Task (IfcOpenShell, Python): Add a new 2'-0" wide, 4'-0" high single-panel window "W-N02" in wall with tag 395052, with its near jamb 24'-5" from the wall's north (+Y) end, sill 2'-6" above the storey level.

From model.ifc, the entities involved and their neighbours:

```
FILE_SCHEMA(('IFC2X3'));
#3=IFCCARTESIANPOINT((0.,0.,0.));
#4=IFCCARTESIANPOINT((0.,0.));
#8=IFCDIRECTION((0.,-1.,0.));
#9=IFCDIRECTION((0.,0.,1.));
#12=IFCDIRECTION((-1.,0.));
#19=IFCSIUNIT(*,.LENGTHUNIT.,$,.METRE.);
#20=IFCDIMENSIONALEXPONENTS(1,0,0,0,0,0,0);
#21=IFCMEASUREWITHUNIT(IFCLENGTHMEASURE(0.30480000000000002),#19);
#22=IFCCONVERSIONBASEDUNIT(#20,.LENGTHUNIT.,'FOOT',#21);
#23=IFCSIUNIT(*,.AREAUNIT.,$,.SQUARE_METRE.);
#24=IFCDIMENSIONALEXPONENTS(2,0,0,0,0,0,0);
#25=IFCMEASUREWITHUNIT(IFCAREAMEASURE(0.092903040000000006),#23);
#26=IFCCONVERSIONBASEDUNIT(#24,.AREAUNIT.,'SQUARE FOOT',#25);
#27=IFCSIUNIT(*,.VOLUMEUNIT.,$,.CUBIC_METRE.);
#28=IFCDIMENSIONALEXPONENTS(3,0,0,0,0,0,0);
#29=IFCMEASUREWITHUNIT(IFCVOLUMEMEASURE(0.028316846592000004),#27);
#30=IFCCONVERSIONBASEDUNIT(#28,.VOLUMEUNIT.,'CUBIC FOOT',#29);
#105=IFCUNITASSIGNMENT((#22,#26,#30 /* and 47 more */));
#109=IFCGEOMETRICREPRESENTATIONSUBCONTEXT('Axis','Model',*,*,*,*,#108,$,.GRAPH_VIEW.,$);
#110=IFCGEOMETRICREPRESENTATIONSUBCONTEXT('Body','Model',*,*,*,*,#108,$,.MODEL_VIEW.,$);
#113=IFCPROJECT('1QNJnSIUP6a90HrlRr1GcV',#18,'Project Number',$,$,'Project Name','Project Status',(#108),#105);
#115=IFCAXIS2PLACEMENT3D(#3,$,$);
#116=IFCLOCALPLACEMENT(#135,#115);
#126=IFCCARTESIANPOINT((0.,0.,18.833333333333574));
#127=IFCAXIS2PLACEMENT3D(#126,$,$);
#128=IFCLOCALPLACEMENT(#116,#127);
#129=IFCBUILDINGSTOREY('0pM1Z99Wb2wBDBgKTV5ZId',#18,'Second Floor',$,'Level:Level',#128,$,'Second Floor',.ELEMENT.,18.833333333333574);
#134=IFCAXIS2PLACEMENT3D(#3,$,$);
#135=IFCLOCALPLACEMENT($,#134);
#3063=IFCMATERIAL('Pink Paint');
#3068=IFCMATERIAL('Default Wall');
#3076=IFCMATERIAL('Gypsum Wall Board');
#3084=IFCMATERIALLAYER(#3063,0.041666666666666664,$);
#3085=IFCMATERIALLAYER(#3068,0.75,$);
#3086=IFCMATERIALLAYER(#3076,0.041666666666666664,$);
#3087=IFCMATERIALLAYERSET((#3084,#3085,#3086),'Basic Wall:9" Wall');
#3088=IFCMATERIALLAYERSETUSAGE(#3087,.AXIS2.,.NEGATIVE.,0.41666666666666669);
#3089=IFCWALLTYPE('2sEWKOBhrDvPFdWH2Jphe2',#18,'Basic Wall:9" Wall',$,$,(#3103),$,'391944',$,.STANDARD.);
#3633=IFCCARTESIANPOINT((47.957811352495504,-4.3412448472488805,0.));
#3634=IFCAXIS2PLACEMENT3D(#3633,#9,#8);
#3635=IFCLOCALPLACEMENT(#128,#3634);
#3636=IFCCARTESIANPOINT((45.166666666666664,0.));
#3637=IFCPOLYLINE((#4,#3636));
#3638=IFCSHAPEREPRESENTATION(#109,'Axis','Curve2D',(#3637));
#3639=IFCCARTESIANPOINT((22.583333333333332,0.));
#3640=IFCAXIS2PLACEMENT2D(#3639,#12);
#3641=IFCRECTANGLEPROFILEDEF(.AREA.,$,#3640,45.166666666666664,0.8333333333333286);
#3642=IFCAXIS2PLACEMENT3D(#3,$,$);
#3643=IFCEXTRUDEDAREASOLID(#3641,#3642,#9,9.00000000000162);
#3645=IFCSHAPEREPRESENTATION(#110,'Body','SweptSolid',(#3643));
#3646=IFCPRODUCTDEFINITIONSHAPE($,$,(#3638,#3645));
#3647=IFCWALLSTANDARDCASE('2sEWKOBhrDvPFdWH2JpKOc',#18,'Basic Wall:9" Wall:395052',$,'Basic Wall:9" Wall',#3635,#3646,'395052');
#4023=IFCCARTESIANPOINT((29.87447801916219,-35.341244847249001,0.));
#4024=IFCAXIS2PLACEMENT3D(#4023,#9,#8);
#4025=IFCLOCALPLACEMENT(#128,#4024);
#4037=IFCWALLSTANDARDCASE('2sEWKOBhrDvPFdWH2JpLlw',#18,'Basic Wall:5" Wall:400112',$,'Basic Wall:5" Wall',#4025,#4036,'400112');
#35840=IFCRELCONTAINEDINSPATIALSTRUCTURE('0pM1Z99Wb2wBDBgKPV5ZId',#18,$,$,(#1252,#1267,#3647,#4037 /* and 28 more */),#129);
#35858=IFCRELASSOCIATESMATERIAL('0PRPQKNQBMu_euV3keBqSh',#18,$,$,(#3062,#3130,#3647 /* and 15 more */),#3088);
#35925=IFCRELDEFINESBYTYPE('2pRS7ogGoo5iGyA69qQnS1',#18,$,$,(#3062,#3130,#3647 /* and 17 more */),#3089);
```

```python
import numpy as np
import ifcopenshell
import ifcopenshell.api.feature
import ifcopenshell.api.geometry
import ifcopenshell.api.root
import ifcopenshell.api.spatial
import ifcopenshell.api.type
import ifcopenshell.geom
import ifcopenshell.util.element
import ifcopenshell.util.placement
import ifcopenshell.util.representation
import ifcopenshell.util.shape
import ifcopenshell.util.unit

model = ifcopenshell.open("model.ifc")
unit_scale = ifcopenshell.util.unit.calculate_unit_scale(model)
settings = ifcopenshell.geom.settings()


def volume(element):
    """Net volume in cubic metres, openings subtracted."""
    shape = ifcopenshell.geom.create_shape(settings, element)
    return ifcopenshell.util.shape.get_volume(shape.geometry)


wall = model.by_guid("2sEWKOBhrDvPFdWH2JpKOc")
storey = ifcopenshell.util.element.get_container(wall, ifc_class="IfcBuildingStorey")
context = ifcopenshell.util.representation.get_context(model, "Model", "Body", "MODEL_VIEW")
before = volume(wall)

width, height, from_end, sill = 0.6096, 1.2192, 7.4422, 0.762  # metres

# The wall runs along its own X axis, and the end named is its -X end.
wall_shape = ifcopenshell.geom.create_shape(settings, wall)
x, y, z = ifcopenshell.util.shape.get_vertices(wall_shape.geometry).T
start = x.min() + from_end
face, thickness = float(y.min()), float(y.max() - y.min())
wall_matrix = ifcopenshell.util.placement.get_local_placement(wall.ObjectPlacement)
level = ifcopenshell.util.placement.get_local_placement(storey.ObjectPlacement)[2, 3]


def in_wall(x, y):
    """Placement at x, y metres in the wall's axes, at sill height."""
    matrix = wall_matrix.copy()
    matrix[:, 3] = wall_matrix @ np.array([x / unit_scale, y / unit_scale, 0.0, 1.0])
    matrix[2, 3] = level + sill / unit_scale
    return matrix


# Opening: a box that overshoots both wall faces by 50 mm.
opening = ifcopenshell.api.root.create_entity(model, ifc_class="IfcOpeningElement")
box = ifcopenshell.api.geometry.add_wall_representation(
    model, context=context, length=width, height=height, thickness=thickness + 0.1
)
ifcopenshell.api.geometry.assign_representation(model, product=opening, representation=box)
ifcopenshell.api.geometry.edit_object_placement(model, product=opening, matrix=in_wall(start, face - 0.05), is_si=False)
ifcopenshell.api.feature.add_feature(model, feature=opening, element=wall)

window = ifcopenshell.api.root.create_entity(model, ifc_class="IfcWindow", name="W-N02")
window.OverallWidth, window.OverallHeight = width / unit_scale, height / unit_scale
body = ifcopenshell.api.geometry.add_window_representation(
    model,
    context=context,
    overall_width=window.OverallWidth,
    overall_height=window.OverallHeight,
    partition_type="SINGLE_PANEL",
)
ifcopenshell.api.geometry.assign_representation(model, product=window, representation=body)
ifcopenshell.api.spatial.assign_container(model, products=[window], relating_structure=storey)
fills = ifcopenshell.api.feature.add_filling(model, opening=opening, element=window)
fills.OwnerHistory = window.OwnerHistory  # required in IFC2X3

# IFC2X3 keeps the operation on the window style.
style = ifcopenshell.api.root.create_entity(model, ifc_class="IfcWindowStyle", name="W-N02")
style.OperationType, style.ConstructionType = "SINGLE_PANEL", "NOTDEFINED"
style.ParameterTakesPrecedence = style.Sizeable = False
ifcopenshell.api.type.assign_type(model, related_objects=[window], relating_type=style)

# Centre the window in the wall's thickness.
ifcopenshell.api.geometry.edit_object_placement(model, product=window, matrix=in_wall(start, face), is_si=False)
window_shape = ifcopenshell.geom.create_shape(settings, window)
depth = ifcopenshell.util.shape.get_vertices(window_shape.geometry)[:, 1]
offset = face + thickness / 2 - (depth.min() + depth.max()) / 2
ifcopenshell.api.geometry.edit_object_placement(model, product=window, matrix=in_wall(start, offset), is_si=False)

after = volume(wall)

print(f"wall volume {before:.3f} -> {after:.3f} m3")

model.write("model_rev.ifc")
```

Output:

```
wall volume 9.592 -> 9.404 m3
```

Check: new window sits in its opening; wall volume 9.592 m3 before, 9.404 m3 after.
